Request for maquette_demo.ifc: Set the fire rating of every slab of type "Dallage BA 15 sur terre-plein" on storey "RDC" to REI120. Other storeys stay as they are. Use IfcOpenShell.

First a look at what the model holds.

```python
import ifcopenshell
import ifcopenshell.util.element

model = ifcopenshell.open("maquette_demo.ifc")
print(model.schema)
storey = next(s for s in model.by_type("IfcBuildingStorey") if s.Name == "RDC")
slabs = [e for e in ifcopenshell.util.element.get_decomposition(storey) if e.is_a("IfcSlab")]
seen = {}
for e in slabs:
    element_type = ifcopenshell.util.element.get_type(e)
    key = (element_type.Name if element_type != e and element_type else None, ifcopenshell.util.element.get_pset(e, "Pset_SlabCommon", "FireRating"))
    seen[key] = seen.get(key, 0) + 1
for (name, value), count in sorted(seen.items(), key=str):
    print(count, "x", name, "|", value)
```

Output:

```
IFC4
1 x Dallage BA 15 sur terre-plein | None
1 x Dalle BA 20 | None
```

```python
import ifcopenshell
import ifcopenshell.api.pset
import ifcopenshell.util.element

model = ifcopenshell.open("maquette_demo.ifc")

storey = next(s for s in model.by_type("IfcBuildingStorey") if s.Name == "RDC")
slabs = [e for e in ifcopenshell.util.element.get_decomposition(storey) if e.is_a("IfcSlab")]

count = 0
for e in slabs:
    element_type = ifcopenshell.util.element.get_type(e)
    if element_type in (None, e) or element_type.Name != "Dallage BA 15 sur terre-plein":
        continue
    # add_pset returns the element's existing set when there is one.
    pset = ifcopenshell.api.pset.add_pset(model, product=e, name="Pset_SlabCommon")
    ifcopenshell.api.pset.edit_pset(model, pset=pset, properties={"FireRating": "REI120"})
    count += 1

print(count, "slabs updated")

model.write("maquette_demo_rev.ifc")
```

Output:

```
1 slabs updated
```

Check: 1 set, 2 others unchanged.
